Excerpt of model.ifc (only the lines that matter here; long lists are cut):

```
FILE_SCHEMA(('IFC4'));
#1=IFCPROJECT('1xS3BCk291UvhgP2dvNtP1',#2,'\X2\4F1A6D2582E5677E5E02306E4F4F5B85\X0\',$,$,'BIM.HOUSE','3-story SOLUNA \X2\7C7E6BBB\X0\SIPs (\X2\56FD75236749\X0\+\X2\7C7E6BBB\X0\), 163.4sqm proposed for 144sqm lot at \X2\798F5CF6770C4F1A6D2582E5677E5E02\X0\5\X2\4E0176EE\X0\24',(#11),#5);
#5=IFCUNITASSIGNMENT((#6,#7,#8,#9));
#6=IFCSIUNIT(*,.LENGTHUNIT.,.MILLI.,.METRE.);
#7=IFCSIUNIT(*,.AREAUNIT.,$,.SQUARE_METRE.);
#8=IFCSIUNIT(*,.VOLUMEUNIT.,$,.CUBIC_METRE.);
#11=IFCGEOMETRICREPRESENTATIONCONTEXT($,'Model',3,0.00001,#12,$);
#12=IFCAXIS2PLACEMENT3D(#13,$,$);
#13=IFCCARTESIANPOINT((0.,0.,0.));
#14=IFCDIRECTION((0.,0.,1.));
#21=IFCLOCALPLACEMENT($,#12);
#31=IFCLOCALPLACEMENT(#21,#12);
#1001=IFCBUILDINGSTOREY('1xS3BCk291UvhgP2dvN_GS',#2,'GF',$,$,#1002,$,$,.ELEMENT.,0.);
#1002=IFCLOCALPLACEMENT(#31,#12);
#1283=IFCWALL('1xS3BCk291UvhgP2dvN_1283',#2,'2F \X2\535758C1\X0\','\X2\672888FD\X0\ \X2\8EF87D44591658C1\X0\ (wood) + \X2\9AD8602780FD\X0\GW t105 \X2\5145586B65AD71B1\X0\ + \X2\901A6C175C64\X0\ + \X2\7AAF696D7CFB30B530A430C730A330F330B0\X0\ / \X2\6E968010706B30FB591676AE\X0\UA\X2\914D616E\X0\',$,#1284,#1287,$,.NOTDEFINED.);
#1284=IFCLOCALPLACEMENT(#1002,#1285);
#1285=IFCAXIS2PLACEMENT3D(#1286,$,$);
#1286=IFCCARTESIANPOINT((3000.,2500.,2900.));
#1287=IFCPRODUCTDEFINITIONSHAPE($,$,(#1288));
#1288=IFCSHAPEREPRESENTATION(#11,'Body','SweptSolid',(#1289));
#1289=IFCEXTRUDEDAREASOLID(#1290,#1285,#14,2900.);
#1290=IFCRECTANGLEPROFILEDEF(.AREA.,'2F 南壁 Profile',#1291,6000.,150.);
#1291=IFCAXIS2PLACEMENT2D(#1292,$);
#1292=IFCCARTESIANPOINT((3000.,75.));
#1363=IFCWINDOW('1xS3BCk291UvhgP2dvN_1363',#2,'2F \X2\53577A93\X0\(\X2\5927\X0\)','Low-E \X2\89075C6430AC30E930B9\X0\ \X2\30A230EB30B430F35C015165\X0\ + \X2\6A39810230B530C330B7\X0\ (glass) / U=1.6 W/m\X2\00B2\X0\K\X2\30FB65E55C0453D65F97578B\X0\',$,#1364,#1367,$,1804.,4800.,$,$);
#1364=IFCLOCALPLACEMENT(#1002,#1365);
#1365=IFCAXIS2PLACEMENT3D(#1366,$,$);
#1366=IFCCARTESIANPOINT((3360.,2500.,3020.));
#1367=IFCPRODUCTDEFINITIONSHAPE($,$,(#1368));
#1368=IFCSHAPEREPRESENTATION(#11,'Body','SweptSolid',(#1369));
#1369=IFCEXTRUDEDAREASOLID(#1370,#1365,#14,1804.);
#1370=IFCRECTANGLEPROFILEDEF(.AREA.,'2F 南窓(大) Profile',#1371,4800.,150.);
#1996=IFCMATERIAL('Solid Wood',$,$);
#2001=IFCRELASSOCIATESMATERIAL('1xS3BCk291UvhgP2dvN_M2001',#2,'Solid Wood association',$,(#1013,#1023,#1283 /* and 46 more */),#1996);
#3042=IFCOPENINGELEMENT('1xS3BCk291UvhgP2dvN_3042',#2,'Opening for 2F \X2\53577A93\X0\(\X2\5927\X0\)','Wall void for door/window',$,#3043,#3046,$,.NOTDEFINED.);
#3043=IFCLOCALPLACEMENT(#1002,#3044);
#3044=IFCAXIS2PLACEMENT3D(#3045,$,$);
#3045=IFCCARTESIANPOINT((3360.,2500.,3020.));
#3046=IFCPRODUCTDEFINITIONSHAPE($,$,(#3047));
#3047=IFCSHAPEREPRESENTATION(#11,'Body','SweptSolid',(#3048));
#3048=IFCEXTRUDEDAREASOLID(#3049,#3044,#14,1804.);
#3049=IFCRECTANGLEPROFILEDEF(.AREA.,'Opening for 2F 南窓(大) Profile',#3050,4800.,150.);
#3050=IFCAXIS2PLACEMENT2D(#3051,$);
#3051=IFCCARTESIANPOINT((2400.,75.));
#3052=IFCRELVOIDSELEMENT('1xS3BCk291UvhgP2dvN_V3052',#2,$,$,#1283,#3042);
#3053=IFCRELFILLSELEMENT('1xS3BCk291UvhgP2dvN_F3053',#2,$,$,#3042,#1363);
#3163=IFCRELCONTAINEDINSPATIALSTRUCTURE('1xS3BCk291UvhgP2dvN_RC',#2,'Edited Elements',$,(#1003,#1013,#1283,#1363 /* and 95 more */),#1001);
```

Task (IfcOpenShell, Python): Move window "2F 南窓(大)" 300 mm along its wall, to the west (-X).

```python
import ifcopenshell
import ifcopenshell.api.geometry
import ifcopenshell.util.placement

model = ifcopenshell.open("model.ifc")

window = model.by_guid("1xS3BCk291UvhgP2dvN_1363")
opening = window.FillsVoids[0].RelatingOpeningElement
wall = opening.VoidsElements[0].RelatingBuildingElement

wall_matrix = ifcopenshell.util.placement.get_local_placement(wall.ObjectPlacement)
shift = wall_matrix[:3, 0] * -300.0
before = ifcopenshell.util.placement.get_local_placement(window.ObjectPlacement)[:3, 3].copy()

# The window is not placed relative to its opening, so move both.
for product in (opening, window):
    matrix = ifcopenshell.util.placement.get_local_placement(product.ObjectPlacement)
    matrix[:3, 3] += shift
    ifcopenshell.api.geometry.edit_object_placement(model, product=product, matrix=matrix, is_si=False)

after = ifcopenshell.util.placement.get_local_placement(window.ObjectPlacement)[:3, 3]
print("window moved by", (after - before).round(3) + 0.0)

model.write("model-out.ifc")
```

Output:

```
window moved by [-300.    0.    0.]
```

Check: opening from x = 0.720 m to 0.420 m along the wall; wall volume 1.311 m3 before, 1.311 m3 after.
